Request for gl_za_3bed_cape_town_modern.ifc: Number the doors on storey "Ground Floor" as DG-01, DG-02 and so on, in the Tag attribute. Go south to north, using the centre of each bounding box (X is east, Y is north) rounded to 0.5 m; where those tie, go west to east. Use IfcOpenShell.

First a look at what the model holds.

```python
import ifcopenshell
import ifcopenshell.util.element
import ifcopenshell.util.placement

model = ifcopenshell.open("gl_za_3bed_cape_town_modern.ifc")
print(model.schema)
storey = next(s for s in model.by_type("IfcBuildingStorey") if s.Name == "Ground Floor")
doors = [e for e in ifcopenshell.util.element.get_decomposition(storey) if e.is_a("IfcDoor")]
for e in sorted(doors, key=lambda e: e.id()):
    origin = ifcopenshell.util.placement.get_local_placement(e.ObjectPlacement)[:3, 3]
    print(e.id(), e.Tag, e.Name, origin.round(2) + 0.0, sep=" | ")
```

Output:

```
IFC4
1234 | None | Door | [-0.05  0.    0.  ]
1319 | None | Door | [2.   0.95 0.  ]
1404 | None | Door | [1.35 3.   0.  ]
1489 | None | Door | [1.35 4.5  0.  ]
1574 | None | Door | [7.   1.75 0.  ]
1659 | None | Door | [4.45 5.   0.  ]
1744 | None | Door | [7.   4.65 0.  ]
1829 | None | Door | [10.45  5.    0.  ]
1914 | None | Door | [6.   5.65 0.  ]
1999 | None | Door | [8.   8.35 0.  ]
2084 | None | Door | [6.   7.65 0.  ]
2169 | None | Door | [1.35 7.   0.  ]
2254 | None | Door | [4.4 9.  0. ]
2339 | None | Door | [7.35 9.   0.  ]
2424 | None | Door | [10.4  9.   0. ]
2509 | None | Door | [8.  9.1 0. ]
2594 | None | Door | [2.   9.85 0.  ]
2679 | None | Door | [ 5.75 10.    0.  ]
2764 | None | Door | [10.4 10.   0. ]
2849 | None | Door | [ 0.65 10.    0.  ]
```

```python
import ifcopenshell
import ifcopenshell.geom
import ifcopenshell.util.element
import ifcopenshell.util.shape

model = ifcopenshell.open("gl_za_3bed_cape_town_modern.ifc")
settings = ifcopenshell.geom.settings()
settings.set("use-world-coords", True)


def centre(element):
    shape = ifcopenshell.geom.create_shape(settings, element)
    return ifcopenshell.util.shape.get_bbox_centroid(shape.geometry)


storey = next(s for s in model.by_type("IfcBuildingStorey") if s.Name == "Ground Floor")
doors = [e for e in ifcopenshell.util.element.get_decomposition(storey) if e.is_a("IfcDoor")]

# Insertion points can sit at a corner or the storey origin, so sort by the geometry (in metres).
centres = {e: centre(e) for e in doors}
doors.sort(key=lambda e: (round(centres[e][1] / 0.5), centres[e][0]))

for i, e in enumerate(doors, start=1):
    number = f"DG-{i:02d}"
    e.Tag = number
    print(e.id(), number)

model.write("gl_za_3bed_cape_town_modern_edited.ifc")
```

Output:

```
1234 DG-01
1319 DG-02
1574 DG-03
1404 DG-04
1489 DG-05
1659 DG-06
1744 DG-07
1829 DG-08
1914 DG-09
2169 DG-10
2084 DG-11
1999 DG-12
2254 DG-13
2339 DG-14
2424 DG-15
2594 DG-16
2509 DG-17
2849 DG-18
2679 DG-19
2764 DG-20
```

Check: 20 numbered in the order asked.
